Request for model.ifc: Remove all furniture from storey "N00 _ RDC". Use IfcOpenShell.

First a look at what the model holds.

```python
import ifcopenshell
import ifcopenshell.util.element

model = ifcopenshell.open("model.ifc")
print(model.schema)
storey = next(s for s in model.by_type("IfcBuildingStorey") if s.Name == "N00 _ RDC")
furniture = [e for e in ifcopenshell.util.element.get_decomposition(storey) if e.is_a("IfcFurnishingElement")]
seen = {}
for e in furniture:
    element_type = ifcopenshell.util.element.get_type(e)
    name = element_type.Name if element_type not in (None, e) else None
    seen[name] = seen.get(name, 0) + 1
for name, count in sorted(seen.items(), key=str):
    print(count, "x", name)
```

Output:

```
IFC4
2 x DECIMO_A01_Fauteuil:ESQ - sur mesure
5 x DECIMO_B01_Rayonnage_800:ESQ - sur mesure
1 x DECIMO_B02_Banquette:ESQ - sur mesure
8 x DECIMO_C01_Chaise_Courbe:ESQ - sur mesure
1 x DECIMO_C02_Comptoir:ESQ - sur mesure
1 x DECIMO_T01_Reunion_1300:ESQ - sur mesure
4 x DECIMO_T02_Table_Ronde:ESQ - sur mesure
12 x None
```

```python
import ifcopenshell
import ifcopenshell.api.root
import ifcopenshell.util.element

model = ifcopenshell.open("model.ifc")

storey = next(s for s in model.by_type("IfcBuildingStorey") if s.Name == "N00 _ RDC")
furniture = [e for e in ifcopenshell.util.element.get_decomposition(storey) if e.is_a("IfcFurnishingElement")]

for e in furniture:
    ifcopenshell.api.root.remove_product(model, product=e)
print(len(furniture), "removed")

model.write("model_v2.ifc")
```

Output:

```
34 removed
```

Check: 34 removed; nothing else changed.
